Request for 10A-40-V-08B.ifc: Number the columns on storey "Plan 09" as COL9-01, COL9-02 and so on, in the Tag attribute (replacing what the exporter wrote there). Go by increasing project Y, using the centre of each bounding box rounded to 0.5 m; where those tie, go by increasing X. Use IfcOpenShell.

First a look at what the model holds.

```python
import ifcopenshell
import ifcopenshell.util.element
import ifcopenshell.util.placement

model = ifcopenshell.open("10A-40-V-08B.ifc")
print(model.schema)
storey = next(s for s in model.by_type("IfcBuildingStorey") if s.Name == "Plan 09")
columns = [e for e in ifcopenshell.util.element.get_decomposition(storey) if e.is_a("IfcColumn")]
for e in sorted(columns, key=lambda e: e.id()):
    origin = ifcopenshell.util.placement.get_local_placement(e.ObjectPlacement)[:3, 3]
    print(e.id(), e.Tag, e.Name, origin.round(2) + 0.0, sep=" | ")
```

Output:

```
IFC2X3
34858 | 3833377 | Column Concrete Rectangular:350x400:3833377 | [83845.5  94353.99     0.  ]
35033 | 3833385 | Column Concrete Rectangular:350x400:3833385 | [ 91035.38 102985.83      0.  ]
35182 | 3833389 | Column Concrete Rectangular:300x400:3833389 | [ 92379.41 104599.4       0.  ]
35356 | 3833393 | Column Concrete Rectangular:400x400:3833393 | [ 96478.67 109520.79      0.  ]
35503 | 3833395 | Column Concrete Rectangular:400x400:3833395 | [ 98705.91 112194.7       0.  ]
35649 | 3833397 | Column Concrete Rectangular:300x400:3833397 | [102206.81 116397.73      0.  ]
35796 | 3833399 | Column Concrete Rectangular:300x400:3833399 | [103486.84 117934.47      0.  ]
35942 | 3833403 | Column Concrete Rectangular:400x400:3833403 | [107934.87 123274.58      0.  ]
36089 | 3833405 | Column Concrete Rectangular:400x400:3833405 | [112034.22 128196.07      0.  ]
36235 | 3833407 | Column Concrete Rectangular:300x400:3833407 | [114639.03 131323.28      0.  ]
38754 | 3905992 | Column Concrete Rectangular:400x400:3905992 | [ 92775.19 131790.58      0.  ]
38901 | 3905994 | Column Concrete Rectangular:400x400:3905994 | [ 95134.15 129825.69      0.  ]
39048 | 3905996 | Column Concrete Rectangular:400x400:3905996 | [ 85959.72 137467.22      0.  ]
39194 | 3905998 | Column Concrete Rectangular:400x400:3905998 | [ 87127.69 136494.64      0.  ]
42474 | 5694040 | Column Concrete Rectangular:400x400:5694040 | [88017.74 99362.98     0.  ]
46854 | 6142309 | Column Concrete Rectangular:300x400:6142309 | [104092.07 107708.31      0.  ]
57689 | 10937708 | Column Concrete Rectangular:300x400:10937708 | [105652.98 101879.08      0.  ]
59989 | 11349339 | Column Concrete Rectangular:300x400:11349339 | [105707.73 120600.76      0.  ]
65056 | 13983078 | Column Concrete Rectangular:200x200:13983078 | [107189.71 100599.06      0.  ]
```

```python
import ifcopenshell
import ifcopenshell.geom
import ifcopenshell.util.element
import ifcopenshell.util.shape

model = ifcopenshell.open("10A-40-V-08B.ifc")
settings = ifcopenshell.geom.settings()
settings.set("use-world-coords", True)


def centre(element):
    shape = ifcopenshell.geom.create_shape(settings, element)
    return ifcopenshell.util.shape.get_bbox_centroid(shape.geometry)


storey = next(s for s in model.by_type("IfcBuildingStorey") if s.Name == "Plan 09")
columns = [e for e in ifcopenshell.util.element.get_decomposition(storey) if e.is_a("IfcColumn")]

# Insertion points can sit at a corner or the storey origin, so sort by the geometry (in metres).
centres = {e: centre(e) for e in columns}
columns.sort(key=lambda e: (round(centres[e][1] / 0.5), centres[e][0]))

for i, e in enumerate(columns, start=1):
    number = f"COL9-{i:02d}"
    e.Tag = number
    print(e.id(), number)

model.write("10A-40-V-08B_edited.ifc")
```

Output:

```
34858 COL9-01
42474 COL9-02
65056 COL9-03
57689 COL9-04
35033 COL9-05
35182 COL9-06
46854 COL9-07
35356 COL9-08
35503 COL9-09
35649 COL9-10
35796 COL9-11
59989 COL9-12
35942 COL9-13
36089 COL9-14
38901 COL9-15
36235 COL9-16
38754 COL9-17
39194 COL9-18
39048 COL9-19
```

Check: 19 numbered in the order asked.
